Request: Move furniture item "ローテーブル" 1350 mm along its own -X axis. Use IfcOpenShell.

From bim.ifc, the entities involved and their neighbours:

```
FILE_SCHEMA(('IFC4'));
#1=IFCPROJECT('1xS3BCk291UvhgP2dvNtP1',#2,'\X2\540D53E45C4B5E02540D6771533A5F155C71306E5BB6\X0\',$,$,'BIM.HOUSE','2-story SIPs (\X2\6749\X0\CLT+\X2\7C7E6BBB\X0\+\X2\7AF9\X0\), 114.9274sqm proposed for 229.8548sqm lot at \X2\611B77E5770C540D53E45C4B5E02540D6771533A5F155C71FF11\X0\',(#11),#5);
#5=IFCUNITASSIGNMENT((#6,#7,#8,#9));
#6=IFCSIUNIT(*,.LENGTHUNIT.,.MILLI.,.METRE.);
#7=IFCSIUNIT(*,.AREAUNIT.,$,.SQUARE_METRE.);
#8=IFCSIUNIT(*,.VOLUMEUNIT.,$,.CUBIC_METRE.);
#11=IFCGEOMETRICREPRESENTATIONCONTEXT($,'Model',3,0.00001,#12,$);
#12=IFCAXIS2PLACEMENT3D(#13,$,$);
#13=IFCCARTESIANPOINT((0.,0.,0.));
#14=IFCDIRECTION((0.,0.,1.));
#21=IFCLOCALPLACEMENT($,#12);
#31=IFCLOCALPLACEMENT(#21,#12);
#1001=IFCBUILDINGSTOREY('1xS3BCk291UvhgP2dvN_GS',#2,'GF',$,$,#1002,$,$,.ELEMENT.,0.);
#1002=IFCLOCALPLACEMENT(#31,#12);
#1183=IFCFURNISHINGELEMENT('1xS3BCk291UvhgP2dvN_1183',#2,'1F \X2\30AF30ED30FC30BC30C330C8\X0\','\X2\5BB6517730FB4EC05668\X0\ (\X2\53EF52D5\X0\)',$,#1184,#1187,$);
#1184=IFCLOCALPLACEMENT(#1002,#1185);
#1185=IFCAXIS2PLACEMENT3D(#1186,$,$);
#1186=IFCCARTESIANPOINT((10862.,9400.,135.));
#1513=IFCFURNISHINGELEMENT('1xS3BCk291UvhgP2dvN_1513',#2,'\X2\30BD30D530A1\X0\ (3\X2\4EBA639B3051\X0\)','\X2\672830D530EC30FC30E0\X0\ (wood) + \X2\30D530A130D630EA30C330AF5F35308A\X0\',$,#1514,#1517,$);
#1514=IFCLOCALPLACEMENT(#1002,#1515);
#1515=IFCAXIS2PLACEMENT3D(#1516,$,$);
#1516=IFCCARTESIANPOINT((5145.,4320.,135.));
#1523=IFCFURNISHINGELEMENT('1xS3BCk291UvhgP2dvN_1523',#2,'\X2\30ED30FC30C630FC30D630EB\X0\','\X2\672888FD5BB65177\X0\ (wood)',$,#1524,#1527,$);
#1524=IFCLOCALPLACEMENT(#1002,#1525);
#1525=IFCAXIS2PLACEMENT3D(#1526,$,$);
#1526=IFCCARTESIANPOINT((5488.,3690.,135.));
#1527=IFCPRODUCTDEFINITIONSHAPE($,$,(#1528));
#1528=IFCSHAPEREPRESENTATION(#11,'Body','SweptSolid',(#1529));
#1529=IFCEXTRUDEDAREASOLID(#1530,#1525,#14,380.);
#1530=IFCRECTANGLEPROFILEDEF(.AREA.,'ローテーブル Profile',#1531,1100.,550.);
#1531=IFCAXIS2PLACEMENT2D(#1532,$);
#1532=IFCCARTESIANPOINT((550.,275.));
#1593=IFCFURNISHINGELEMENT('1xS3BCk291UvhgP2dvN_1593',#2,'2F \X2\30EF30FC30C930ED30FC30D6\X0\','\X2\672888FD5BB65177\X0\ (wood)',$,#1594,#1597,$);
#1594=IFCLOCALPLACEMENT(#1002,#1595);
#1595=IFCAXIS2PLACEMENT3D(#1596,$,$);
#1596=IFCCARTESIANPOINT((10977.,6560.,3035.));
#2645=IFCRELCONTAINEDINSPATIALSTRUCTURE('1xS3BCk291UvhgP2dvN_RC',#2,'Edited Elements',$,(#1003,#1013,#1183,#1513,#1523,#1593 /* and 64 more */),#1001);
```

```python
import ifcopenshell
import ifcopenshell.api.geometry
import ifcopenshell.util.placement
import ifcopenshell.util.unit

model = ifcopenshell.open("bim.ifc")
unit_scale = ifcopenshell.util.unit.calculate_unit_scale(model)

item = model.by_guid("1xS3BCk291UvhgP2dvN_1523")
matrix = ifcopenshell.util.placement.get_local_placement(item.ObjectPlacement)
matrix[:3, 3] -= matrix[:3, 0] * 1.35 / unit_scale
ifcopenshell.api.geometry.edit_object_placement(model, product=item, matrix=matrix, is_si=False)

print(ifcopenshell.util.placement.get_local_placement(item.ObjectPlacement).round(3) + 0.0)

model.write("bim_rev.ifc")
```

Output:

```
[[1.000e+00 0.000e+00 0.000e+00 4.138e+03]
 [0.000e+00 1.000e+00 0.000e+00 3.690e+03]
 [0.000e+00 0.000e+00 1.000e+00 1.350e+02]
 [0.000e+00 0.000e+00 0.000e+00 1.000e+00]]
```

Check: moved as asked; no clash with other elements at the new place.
